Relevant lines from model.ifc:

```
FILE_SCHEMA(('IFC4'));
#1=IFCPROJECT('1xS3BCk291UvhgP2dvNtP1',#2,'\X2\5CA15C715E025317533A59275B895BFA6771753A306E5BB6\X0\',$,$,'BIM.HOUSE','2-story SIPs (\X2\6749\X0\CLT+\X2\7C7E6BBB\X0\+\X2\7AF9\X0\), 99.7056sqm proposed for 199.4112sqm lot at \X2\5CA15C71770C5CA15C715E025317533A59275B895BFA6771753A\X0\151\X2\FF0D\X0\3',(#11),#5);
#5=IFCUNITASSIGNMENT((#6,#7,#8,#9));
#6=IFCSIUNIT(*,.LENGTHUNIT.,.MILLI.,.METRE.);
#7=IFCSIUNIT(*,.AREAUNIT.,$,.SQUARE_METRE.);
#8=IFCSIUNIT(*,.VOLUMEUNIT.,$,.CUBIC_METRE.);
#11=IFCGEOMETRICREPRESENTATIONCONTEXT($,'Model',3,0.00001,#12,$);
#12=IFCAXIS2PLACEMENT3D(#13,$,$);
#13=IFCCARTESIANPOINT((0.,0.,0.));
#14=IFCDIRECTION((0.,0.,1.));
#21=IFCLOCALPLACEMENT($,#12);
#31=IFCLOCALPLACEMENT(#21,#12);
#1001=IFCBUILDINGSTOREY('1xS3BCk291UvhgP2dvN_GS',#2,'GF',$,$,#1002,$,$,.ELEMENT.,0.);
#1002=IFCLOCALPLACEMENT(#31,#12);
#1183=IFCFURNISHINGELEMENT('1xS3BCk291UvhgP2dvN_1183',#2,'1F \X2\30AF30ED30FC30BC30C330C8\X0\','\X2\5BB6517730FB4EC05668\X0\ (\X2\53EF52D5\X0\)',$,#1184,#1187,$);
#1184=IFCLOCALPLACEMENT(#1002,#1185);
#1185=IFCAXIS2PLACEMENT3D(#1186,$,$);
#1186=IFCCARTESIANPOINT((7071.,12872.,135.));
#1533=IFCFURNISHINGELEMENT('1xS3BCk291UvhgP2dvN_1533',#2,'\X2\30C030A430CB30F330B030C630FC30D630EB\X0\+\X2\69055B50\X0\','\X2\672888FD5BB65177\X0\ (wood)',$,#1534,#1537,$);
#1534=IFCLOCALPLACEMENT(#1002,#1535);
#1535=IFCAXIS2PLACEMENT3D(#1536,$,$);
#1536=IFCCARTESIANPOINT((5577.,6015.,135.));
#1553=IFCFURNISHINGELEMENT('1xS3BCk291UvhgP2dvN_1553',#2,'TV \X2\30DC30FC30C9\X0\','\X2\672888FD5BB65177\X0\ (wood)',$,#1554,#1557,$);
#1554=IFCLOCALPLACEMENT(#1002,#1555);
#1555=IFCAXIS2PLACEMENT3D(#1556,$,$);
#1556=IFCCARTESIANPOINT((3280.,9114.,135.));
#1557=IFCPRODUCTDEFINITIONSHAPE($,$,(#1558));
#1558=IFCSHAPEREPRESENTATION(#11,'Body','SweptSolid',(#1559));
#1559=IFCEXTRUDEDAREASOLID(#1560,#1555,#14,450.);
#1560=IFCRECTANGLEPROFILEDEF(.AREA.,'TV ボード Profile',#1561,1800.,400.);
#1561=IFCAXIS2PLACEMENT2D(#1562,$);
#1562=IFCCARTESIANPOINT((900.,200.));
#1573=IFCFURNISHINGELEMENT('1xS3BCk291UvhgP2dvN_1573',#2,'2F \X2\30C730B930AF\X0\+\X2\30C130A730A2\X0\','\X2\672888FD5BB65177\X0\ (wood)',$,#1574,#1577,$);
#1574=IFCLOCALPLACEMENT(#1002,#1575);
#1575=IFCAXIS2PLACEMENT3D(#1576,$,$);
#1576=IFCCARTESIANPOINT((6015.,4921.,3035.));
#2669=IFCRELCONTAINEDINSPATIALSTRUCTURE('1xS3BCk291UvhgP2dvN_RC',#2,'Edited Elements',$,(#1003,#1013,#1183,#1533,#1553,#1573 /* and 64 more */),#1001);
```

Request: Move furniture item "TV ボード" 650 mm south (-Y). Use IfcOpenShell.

```python
import ifcopenshell
import ifcopenshell.api.geometry
import ifcopenshell.util.placement
import ifcopenshell.util.unit

model = ifcopenshell.open("model.ifc")
unit_scale = ifcopenshell.util.unit.calculate_unit_scale(model)

item = model.by_guid("1xS3BCk291UvhgP2dvN_1553")
matrix = ifcopenshell.util.placement.get_local_placement(item.ObjectPlacement)
matrix[1, 3] -= 0.65 / unit_scale
ifcopenshell.api.geometry.edit_object_placement(model, product=item, matrix=matrix, is_si=False)

print(ifcopenshell.util.placement.get_local_placement(item.ObjectPlacement).round(3) + 0.0)

model.write("model_v2.ifc")
```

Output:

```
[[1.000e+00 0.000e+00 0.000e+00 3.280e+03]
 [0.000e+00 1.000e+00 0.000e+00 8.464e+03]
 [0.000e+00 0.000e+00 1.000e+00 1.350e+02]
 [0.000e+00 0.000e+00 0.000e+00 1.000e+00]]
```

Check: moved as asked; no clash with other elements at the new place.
